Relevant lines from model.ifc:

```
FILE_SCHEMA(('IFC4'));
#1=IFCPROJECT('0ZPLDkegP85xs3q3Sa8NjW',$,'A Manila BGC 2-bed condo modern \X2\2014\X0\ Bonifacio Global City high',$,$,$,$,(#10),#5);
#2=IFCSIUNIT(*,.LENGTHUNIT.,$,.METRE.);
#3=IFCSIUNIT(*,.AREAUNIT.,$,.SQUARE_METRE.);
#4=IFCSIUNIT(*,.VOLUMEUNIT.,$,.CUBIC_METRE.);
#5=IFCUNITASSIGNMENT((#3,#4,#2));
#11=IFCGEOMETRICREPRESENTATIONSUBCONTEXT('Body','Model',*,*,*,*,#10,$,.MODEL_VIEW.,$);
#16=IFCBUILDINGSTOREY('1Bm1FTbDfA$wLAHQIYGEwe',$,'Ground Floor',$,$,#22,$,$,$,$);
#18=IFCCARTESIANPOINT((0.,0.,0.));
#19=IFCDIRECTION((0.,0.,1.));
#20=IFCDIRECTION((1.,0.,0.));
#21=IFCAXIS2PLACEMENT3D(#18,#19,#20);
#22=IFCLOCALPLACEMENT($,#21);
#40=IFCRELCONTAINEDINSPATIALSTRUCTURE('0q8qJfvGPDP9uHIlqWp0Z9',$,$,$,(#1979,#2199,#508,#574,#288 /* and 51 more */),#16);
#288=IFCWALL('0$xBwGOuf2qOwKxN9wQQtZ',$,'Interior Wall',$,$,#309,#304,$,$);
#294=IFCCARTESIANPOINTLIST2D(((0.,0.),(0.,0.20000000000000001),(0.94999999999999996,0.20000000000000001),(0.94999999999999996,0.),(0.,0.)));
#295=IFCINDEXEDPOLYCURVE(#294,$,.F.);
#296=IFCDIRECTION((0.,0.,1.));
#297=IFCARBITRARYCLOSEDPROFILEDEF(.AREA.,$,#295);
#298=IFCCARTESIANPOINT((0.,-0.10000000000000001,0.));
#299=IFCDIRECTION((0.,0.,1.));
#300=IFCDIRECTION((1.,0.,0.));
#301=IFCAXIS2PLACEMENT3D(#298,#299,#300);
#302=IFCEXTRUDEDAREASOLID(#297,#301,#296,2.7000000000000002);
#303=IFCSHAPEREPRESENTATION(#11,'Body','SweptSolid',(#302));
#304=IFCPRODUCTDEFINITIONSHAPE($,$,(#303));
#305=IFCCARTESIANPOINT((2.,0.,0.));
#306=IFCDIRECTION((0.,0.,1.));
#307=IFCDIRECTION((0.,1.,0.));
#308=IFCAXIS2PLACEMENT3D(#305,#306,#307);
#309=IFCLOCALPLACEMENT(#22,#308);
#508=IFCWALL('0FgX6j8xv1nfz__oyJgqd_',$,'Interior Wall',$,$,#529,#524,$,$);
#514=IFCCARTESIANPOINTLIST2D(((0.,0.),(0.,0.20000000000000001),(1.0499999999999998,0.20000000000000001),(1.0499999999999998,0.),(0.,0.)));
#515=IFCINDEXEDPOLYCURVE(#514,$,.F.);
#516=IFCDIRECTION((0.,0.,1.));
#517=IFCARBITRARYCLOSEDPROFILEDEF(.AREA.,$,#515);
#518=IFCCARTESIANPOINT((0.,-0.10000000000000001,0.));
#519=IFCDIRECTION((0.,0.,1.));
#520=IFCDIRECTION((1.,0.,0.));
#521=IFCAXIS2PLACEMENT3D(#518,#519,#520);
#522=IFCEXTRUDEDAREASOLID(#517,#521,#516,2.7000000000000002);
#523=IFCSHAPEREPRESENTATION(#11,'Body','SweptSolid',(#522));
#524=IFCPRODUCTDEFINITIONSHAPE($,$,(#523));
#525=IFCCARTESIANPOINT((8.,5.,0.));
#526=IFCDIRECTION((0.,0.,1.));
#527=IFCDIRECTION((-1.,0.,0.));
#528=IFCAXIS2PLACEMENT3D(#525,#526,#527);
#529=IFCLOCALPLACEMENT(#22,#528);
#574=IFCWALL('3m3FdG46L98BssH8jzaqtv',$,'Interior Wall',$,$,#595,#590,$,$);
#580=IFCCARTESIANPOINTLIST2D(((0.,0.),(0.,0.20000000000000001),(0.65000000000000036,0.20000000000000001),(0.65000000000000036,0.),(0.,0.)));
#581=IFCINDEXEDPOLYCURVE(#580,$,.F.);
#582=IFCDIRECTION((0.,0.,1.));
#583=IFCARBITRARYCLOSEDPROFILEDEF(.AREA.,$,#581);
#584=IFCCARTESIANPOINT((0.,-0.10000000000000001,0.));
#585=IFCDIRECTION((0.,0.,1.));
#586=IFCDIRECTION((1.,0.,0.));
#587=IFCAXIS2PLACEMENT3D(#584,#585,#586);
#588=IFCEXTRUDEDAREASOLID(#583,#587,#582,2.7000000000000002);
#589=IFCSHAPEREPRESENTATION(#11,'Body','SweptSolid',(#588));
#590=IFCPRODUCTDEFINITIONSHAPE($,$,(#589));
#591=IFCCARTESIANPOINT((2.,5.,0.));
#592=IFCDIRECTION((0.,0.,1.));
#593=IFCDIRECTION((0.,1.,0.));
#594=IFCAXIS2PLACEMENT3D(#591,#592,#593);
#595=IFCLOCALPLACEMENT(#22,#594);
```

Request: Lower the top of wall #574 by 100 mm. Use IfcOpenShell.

```python
import ifcopenshell
import ifcopenshell.geom
import ifcopenshell.util.representation
import ifcopenshell.util.shape

model = ifcopenshell.open("model.ifc")
settings = ifcopenshell.geom.settings()


def volume(element):
    """Net volume in cubic metres, openings subtracted."""
    shape = ifcopenshell.geom.create_shape(settings, element)
    return ifcopenshell.util.shape.get_volume(shape.geometry)


wall = model.by_guid("3m3FdG46L98BssH8jzaqtv")
before = volume(wall)

body = ifcopenshell.util.representation.get_representation(wall, "Model", "Body")
solid = body.Items[0]
old_height = solid.Depth
solid.Depth -= 0.1
after = volume(wall)

print(f"height {old_height:g} -> {solid.Depth:g}, volume {before:.3f} -> {after:.3f} m3")

model.write("model_rev.ifc")
```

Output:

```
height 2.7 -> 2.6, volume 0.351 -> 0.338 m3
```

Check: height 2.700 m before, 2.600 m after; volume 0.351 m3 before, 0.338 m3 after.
